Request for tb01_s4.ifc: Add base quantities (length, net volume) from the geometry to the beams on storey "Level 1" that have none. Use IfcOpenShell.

First a look at what the model holds.

```python
import ifcopenshell
import ifcopenshell.util.element
import ifcopenshell.util.unit

model = ifcopenshell.open("tb01_s4.ifc")
print(model.schema)
for unit_type in ("LENGTHUNIT", "AREAUNIT", "VOLUMEUNIT"):
    print(unit_type, ifcopenshell.util.unit.calculate_unit_scale(model, unit_type))
storey = next(s for s in model.by_type("IfcBuildingStorey") if s.Name == "Level 1")
beams = [e for e in ifcopenshell.util.element.get_decomposition(storey) if e.is_a("IfcBeam")]
for e in sorted(beams, key=lambda e: e.id()):
    print(e.id(), e.is_a(), e.Name, list(ifcopenshell.util.element.get_psets(e, qtos_only=True)), sep=" | ")
```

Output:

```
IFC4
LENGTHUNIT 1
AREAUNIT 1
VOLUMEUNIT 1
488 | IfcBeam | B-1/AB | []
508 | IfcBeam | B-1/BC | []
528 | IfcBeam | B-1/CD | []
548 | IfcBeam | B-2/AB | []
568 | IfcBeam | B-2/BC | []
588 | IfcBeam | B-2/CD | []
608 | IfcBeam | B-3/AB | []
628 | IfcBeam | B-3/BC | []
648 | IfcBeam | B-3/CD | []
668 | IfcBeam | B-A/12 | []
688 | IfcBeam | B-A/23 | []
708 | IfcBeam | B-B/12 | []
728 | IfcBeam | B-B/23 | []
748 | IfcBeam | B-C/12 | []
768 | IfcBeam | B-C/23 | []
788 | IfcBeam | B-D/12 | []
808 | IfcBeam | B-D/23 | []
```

```python
import ifcopenshell
import ifcopenshell.api.pset
import ifcopenshell.geom
import ifcopenshell.util.element
import ifcopenshell.util.shape
import ifcopenshell.util.unit

model = ifcopenshell.open("tb01_s4.ifc")
unit_scale = ifcopenshell.util.unit.calculate_unit_scale(model)
volume_scale = ifcopenshell.util.unit.calculate_unit_scale(model, "VOLUMEUNIT")
settings = ifcopenshell.geom.settings()

storey = next(s for s in model.by_type("IfcBuildingStorey") if s.Name == "Level 1")
beams = [e for e in ifcopenshell.util.element.get_decomposition(storey) if e.is_a("IfcBeam")]

for e in sorted(beams, key=lambda e: e.id()):
    if ifcopenshell.util.element.get_psets(e, qtos_only=True, should_inherit=False):
        continue
    # Geometry comes back in metres, in the element's own axes.
    shape = ifcopenshell.geom.create_shape(settings, e)
    values = {
        "Length": ifcopenshell.util.shape.get_max_xyz(shape.geometry) / unit_scale,
        "NetVolume": ifcopenshell.util.shape.get_volume(shape.geometry) / volume_scale,
    }
    qto = ifcopenshell.api.pset.add_qto(model, product=e, name="Qto_BeamBaseQuantities")
    ifcopenshell.api.pset.edit_qto(model, qto=qto, properties=values)
    print(e.id(), {k: round(v, 3) for k, v in values.items()})

model.write("tb01_s4_updated.ifc")
```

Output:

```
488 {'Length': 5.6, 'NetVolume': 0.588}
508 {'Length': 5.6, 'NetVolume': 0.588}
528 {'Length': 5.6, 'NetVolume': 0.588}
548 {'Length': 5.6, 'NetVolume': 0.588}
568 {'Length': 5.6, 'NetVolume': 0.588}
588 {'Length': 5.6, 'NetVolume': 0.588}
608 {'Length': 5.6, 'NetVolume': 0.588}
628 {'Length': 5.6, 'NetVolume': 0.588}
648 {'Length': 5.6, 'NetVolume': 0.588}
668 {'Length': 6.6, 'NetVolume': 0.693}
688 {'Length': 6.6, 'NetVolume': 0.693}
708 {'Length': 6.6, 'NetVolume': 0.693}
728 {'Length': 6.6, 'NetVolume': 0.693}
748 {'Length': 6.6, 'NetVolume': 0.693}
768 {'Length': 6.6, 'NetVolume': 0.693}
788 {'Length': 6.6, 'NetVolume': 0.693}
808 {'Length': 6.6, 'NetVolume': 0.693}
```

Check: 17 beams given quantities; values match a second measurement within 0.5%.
